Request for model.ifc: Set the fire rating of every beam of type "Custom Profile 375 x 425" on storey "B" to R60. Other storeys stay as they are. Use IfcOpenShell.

First a look at what the model holds.

```python
import ifcopenshell
import ifcopenshell.util.element

model = ifcopenshell.open("model.ifc")
print(model.schema)
storey = next(s for s in model.by_type("IfcBuildingStorey") if s.Name == "B")
beams = [e for e in ifcopenshell.util.element.get_decomposition(storey) if e.is_a("IfcBeam")]
seen = {}
for e in beams:
    element_type = ifcopenshell.util.element.get_type(e)
    key = (element_type.Name if element_type != e and element_type else None, ifcopenshell.util.element.get_pset(e, "Pset_BeamCommon", "FireRating"))
    seen[key] = seen.get(key, 0) + 1
for (name, value), count in sorted(seen.items(), key=str):
    print(count, "x", name, "|", value)
```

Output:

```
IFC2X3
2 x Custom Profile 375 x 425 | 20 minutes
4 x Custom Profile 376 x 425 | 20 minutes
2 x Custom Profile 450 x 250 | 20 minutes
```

```python
import ifcopenshell
import ifcopenshell.api.pset
import ifcopenshell.util.element

model = ifcopenshell.open("model.ifc")

storey = next(s for s in model.by_type("IfcBuildingStorey") if s.Name == "B")
beams = [e for e in ifcopenshell.util.element.get_decomposition(storey) if e.is_a("IfcBeam")]

count = 0
for e in beams:
    element_type = ifcopenshell.util.element.get_type(e)
    if element_type in (None, e) or element_type.Name != "Custom Profile 375 x 425":
        continue
    # add_pset returns the element's existing set when there is one.
    pset = ifcopenshell.api.pset.add_pset(model, product=e, name="Pset_BeamCommon")
    ifcopenshell.api.pset.edit_pset(model, pset=pset, properties={"FireRating": "R60"})
    count += 1

print(count, "beams updated")

model.write("model_edited.ifc")
```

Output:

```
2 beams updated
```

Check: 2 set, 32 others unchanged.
